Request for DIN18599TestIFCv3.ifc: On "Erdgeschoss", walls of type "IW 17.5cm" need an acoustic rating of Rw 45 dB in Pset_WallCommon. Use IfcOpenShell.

First a look at what the model holds.

```python
import ifcopenshell
import ifcopenshell.util.element

model = ifcopenshell.open("DIN18599TestIFCv3.ifc")
print(model.schema)
storey = next(s for s in model.by_type("IfcBuildingStorey") if s.Name == "Erdgeschoss")
walls = [e for e in ifcopenshell.util.element.get_decomposition(storey) if e.is_a("IfcWall")]
seen = {}
for e in walls:
    element_type = ifcopenshell.util.element.get_type(e)
    key = (element_type.Name if element_type != e and element_type else None, ifcopenshell.util.element.get_pset(e, "Pset_WallCommon", "AcousticRating"))
    seen[key] = seen.get(key, 0) + 1
for (name, value), count in sorted(seen.items(), key=str):
    print(count, "x", name, "|", value)
```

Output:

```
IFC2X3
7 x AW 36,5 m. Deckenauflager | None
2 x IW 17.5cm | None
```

```python
import ifcopenshell
import ifcopenshell.api.pset
import ifcopenshell.util.element

model = ifcopenshell.open("DIN18599TestIFCv3.ifc")

storey = next(s for s in model.by_type("IfcBuildingStorey") if s.Name == "Erdgeschoss")
walls = [e for e in ifcopenshell.util.element.get_decomposition(storey) if e.is_a("IfcWall")]

count = 0
for e in walls:
    element_type = ifcopenshell.util.element.get_type(e)
    if element_type in (None, e) or element_type.Name != "IW 17.5cm":
        continue
    # add_pset returns the element's existing set when there is one.
    pset = ifcopenshell.api.pset.add_pset(model, product=e, name="Pset_WallCommon")
    ifcopenshell.api.pset.edit_pset(model, pset=pset, properties={"AcousticRating": "Rw 45 dB"})
    count += 1

print(count, "walls updated")

model.write("DIN18599TestIFCv3-out.ifc")
```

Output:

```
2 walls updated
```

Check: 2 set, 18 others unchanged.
